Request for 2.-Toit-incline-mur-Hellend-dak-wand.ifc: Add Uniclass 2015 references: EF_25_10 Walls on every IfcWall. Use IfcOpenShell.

First a look at what the model holds.

```python
import ifcopenshell

model = ifcopenshell.open("2.-Toit-incline-mur-Hellend-dak-wand.ifc")
print(model.schema)
print("classifications:", [c.Name for c in model.by_type("IfcClassification")])
for ifc_class in ("IfcDoor", "IfcRoof", "IfcStair", "IfcWall", "IfcWindow"):
    print(ifc_class, len(model.by_type(ifc_class)))
```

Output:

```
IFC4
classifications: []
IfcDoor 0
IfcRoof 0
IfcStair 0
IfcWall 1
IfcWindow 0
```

```python
import ifcopenshell
import ifcopenshell.api.classification

model = ifcopenshell.open("2.-Toit-incline-mur-Hellend-dak-wand.ifc")

system = ifcopenshell.api.classification.add_classification(model, classification="Uniclass 2015")

codes = {
    "IfcWall": ("EF_25_10", "Walls"),
}
for ifc_class, (code, name) in codes.items():
    products = model.by_type(ifc_class)
    ifcopenshell.api.classification.add_reference(
        model, products=products, classification=system, identification=code, name=name
    )
    print(code, len(products))

model.write("2.-Toit-incline-mur-Hellend-dak-wand_rev.ifc")
```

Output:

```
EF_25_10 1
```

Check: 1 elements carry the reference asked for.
